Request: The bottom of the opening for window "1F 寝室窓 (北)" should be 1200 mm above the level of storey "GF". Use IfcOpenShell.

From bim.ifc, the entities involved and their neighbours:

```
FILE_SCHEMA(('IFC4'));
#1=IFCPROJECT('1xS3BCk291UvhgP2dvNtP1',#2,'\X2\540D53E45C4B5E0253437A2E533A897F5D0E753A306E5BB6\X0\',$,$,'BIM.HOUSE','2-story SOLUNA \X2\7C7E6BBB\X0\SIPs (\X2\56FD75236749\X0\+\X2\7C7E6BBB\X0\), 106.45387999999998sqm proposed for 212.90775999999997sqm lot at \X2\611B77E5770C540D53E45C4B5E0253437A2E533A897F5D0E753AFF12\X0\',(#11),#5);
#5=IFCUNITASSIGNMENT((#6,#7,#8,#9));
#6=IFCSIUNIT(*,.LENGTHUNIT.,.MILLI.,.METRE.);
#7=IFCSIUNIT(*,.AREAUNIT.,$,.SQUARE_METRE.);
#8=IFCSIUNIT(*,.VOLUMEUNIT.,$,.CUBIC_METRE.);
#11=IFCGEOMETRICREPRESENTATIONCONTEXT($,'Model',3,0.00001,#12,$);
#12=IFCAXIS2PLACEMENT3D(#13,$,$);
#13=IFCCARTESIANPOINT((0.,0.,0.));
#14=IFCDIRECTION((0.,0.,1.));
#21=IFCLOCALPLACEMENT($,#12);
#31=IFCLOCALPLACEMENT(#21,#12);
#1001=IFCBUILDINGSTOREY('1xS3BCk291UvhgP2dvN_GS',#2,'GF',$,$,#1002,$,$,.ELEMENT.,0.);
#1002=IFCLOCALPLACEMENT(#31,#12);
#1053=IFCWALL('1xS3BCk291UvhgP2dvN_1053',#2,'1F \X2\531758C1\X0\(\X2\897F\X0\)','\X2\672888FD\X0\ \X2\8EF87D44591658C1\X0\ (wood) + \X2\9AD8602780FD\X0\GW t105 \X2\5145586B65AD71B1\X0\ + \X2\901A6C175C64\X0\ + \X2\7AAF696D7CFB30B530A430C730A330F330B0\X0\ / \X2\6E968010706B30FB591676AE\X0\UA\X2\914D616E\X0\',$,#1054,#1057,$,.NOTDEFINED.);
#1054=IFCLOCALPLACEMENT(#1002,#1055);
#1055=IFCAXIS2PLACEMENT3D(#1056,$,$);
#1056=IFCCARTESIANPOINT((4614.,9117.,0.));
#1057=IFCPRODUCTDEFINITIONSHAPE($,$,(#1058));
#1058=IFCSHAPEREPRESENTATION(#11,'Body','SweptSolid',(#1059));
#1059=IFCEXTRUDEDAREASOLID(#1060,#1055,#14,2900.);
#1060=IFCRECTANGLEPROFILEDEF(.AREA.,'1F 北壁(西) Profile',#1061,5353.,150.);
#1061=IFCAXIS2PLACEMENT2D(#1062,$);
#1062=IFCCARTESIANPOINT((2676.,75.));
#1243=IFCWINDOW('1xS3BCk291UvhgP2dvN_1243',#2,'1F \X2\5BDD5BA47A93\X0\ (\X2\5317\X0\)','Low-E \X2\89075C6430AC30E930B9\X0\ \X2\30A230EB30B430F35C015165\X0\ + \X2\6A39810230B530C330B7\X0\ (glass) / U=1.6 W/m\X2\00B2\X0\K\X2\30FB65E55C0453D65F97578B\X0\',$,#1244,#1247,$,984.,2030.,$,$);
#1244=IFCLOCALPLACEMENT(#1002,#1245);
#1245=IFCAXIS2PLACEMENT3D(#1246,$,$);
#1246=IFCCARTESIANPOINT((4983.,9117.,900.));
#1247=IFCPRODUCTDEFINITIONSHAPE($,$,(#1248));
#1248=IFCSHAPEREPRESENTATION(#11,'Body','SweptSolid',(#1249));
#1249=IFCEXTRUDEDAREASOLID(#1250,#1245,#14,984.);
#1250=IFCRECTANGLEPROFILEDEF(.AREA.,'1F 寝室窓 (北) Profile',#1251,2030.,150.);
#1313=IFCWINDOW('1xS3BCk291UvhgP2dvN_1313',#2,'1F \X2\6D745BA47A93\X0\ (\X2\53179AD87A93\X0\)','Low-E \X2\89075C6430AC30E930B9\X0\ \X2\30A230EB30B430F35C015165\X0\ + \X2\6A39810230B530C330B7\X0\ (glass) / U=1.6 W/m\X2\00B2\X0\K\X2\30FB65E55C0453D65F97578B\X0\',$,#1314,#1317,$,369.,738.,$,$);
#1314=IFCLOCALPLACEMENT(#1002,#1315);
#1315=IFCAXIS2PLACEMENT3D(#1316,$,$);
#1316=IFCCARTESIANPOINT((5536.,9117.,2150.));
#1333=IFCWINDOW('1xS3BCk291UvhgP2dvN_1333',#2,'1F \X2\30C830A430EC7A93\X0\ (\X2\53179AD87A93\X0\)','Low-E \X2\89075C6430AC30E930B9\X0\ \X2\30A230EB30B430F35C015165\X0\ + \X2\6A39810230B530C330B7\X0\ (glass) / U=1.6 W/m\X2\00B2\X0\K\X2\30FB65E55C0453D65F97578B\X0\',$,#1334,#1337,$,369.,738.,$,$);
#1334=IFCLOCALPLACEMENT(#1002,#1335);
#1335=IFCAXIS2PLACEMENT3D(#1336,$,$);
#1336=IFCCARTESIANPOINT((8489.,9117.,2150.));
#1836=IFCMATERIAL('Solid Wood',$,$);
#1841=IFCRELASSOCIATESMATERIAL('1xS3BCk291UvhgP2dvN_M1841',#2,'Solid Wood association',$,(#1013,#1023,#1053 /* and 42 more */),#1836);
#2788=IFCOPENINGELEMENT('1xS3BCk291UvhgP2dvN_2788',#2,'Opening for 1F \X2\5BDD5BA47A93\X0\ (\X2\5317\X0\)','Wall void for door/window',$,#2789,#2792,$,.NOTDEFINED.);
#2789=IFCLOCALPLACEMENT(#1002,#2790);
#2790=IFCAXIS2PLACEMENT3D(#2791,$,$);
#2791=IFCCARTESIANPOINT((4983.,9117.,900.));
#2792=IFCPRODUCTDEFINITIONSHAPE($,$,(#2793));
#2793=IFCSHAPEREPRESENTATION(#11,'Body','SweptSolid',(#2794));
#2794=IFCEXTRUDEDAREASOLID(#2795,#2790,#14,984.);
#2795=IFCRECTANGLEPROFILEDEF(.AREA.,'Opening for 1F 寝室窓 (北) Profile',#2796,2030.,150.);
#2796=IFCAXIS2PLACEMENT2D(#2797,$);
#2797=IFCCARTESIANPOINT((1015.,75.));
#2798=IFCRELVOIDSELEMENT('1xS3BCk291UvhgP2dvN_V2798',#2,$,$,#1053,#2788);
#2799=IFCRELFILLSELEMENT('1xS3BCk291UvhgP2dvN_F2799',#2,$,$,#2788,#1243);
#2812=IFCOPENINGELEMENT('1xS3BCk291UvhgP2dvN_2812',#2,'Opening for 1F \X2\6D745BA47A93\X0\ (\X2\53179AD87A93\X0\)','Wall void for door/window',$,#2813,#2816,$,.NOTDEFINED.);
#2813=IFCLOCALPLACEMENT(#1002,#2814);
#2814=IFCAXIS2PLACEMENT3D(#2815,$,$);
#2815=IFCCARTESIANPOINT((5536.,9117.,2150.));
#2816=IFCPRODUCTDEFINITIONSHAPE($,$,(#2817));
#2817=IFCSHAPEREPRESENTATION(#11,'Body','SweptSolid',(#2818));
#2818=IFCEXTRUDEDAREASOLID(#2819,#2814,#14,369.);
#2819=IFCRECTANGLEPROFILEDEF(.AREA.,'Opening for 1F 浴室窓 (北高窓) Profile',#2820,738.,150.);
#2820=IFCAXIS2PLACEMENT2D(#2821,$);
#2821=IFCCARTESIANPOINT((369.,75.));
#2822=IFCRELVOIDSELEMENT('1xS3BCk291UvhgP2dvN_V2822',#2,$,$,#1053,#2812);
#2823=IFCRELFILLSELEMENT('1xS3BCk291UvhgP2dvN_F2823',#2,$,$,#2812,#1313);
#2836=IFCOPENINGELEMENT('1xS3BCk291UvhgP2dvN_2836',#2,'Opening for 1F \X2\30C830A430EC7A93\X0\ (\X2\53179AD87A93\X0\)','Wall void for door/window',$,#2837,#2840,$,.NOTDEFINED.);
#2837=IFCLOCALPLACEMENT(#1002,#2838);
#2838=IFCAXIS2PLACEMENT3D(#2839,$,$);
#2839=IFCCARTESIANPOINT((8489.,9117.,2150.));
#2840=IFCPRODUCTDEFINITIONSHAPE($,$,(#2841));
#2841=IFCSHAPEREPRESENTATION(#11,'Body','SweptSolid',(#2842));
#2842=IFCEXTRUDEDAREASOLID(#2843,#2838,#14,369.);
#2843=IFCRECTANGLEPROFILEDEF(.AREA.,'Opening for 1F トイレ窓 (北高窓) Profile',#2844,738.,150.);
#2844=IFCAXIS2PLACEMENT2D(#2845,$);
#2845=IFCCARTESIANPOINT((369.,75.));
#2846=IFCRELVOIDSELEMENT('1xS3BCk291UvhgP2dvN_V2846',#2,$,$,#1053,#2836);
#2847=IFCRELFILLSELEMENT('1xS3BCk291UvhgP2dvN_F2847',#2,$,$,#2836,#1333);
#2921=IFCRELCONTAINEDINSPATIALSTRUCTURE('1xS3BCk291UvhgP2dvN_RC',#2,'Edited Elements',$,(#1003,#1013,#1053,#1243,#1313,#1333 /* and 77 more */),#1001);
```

```python
import numpy as np
import ifcopenshell
import ifcopenshell.api.geometry
import ifcopenshell.geom
import ifcopenshell.util.element
import ifcopenshell.util.placement
import ifcopenshell.util.shape
import ifcopenshell.util.unit

model = ifcopenshell.open("bim.ifc")
unit_scale = ifcopenshell.util.unit.calculate_unit_scale(model)

window = model.by_guid("1xS3BCk291UvhgP2dvN_1243")
opening = window.FillsVoids[0].RelatingOpeningElement
storey = ifcopenshell.util.element.get_container(window, ifc_class="IfcBuildingStorey")
level = ifcopenshell.util.placement.get_local_placement(storey.ObjectPlacement)[2, 3]

# The opening's origin need not be at the sill, so measure its lowest point.
shape = ifcopenshell.geom.create_shape(ifcopenshell.geom.settings(), opening)
bottom = ifcopenshell.util.shape.get_shape_bottom_elevation(shape, shape.geometry) / unit_scale
dz = level + 1.2 / unit_scale - bottom

shift = np.array([0.0, 0.0, dz])
# The window is not placed relative to its opening, so move both.
for product in (opening, window):
    matrix = ifcopenshell.util.placement.get_local_placement(product.ObjectPlacement)
    matrix[:3, 3] += shift
    ifcopenshell.api.geometry.edit_object_placement(model, product=product, matrix=matrix, is_si=False)

print(f"moved by {dz * unit_scale:+.3f} m")

model.write("bim-out.ifc")
```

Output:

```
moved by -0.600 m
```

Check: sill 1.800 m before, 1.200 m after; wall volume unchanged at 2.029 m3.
